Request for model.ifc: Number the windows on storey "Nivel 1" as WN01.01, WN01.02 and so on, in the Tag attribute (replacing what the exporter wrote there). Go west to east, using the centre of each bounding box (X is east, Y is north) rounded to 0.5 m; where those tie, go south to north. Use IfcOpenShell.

First a look at what the model holds.

```python
import ifcopenshell
import ifcopenshell.util.element
import ifcopenshell.util.placement

model = ifcopenshell.open("model.ifc")
print(model.schema)
storey = next(s for s in model.by_type("IfcBuildingStorey") if s.Name == "Nivel 1")
windows = [e for e in ifcopenshell.util.element.get_decomposition(storey) if e.is_a("IfcWindow")]
for e in sorted(windows, key=lambda e: e.id()):
    origin = ifcopenshell.util.placement.get_local_placement(e.ObjectPlacement)[:3, 3]
    print(e.id(), e.Tag, e.Name, origin.round(2) + 0.0, sep=" | ")
```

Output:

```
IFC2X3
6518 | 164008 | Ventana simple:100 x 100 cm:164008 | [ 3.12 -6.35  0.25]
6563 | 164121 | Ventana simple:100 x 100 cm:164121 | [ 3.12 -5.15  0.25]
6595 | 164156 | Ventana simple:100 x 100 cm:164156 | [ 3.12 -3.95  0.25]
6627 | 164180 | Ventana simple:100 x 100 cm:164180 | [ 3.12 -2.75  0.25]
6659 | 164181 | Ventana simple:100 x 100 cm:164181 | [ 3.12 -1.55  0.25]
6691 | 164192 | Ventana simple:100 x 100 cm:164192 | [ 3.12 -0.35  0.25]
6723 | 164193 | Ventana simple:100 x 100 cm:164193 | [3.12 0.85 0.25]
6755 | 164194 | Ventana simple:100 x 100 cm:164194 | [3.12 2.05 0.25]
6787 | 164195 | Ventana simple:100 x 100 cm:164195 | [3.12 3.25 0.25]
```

```python
import ifcopenshell
import ifcopenshell.geom
import ifcopenshell.util.element
import ifcopenshell.util.shape

model = ifcopenshell.open("model.ifc")
settings = ifcopenshell.geom.settings()
settings.set("use-world-coords", True)


def centre(element):
    shape = ifcopenshell.geom.create_shape(settings, element)
    return ifcopenshell.util.shape.get_bbox_centroid(shape.geometry)


storey = next(s for s in model.by_type("IfcBuildingStorey") if s.Name == "Nivel 1")
windows = [e for e in ifcopenshell.util.element.get_decomposition(storey) if e.is_a("IfcWindow")]

# Insertion points can sit at a corner or the storey origin, so sort by the geometry (in metres).
centres = {e: centre(e) for e in windows}
windows.sort(key=lambda e: (round(centres[e][0] / 0.5), centres[e][1]))

for i, e in enumerate(windows, start=1):
    number = f"WN01.{i:02d}"
    e.Tag = number
    print(e.id(), number)

model.write("model-out.ifc")
```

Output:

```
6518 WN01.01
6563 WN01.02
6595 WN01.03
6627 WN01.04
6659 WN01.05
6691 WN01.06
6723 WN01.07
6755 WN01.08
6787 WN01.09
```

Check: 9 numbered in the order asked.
